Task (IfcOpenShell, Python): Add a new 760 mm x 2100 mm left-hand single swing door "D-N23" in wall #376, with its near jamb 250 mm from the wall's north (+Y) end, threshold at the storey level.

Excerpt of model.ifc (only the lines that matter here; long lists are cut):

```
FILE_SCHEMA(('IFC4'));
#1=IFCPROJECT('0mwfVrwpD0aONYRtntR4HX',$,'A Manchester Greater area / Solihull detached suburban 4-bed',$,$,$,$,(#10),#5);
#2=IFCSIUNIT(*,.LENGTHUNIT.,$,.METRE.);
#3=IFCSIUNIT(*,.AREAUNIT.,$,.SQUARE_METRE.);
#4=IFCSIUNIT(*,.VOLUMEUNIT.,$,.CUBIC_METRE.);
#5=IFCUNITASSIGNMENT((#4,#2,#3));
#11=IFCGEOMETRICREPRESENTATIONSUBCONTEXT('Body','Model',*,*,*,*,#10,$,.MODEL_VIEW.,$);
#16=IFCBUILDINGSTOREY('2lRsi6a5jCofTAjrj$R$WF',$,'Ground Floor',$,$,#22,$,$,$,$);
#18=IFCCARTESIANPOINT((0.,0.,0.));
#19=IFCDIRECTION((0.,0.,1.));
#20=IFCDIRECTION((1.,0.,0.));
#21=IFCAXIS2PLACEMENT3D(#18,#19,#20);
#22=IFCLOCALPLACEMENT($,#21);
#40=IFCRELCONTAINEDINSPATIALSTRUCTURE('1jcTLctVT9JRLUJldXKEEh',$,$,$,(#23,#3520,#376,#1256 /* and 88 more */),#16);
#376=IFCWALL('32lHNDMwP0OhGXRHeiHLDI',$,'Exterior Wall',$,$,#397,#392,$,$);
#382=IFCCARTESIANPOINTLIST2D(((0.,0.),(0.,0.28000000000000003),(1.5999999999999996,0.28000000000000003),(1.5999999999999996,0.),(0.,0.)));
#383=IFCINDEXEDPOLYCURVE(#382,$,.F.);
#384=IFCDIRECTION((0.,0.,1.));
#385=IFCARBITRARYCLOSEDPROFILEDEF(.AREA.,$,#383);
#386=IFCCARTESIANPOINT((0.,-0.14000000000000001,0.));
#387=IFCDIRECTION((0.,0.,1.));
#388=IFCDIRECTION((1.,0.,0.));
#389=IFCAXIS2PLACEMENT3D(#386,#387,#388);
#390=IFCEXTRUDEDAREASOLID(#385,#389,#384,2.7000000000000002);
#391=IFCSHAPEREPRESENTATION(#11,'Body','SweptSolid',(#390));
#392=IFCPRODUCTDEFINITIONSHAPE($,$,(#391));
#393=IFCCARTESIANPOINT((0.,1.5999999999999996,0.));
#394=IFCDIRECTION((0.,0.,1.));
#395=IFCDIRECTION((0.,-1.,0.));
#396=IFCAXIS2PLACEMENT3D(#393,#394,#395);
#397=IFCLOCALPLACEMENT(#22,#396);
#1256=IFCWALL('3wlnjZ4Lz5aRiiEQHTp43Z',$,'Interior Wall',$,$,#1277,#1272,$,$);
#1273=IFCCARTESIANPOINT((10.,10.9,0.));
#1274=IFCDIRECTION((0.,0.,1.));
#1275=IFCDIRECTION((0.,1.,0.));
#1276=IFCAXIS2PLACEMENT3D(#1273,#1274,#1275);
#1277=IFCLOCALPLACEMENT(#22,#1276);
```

```python
import numpy as np
import ifcopenshell
import ifcopenshell.api.feature
import ifcopenshell.api.geometry
import ifcopenshell.api.root
import ifcopenshell.api.spatial
import ifcopenshell.geom
import ifcopenshell.util.element
import ifcopenshell.util.placement
import ifcopenshell.util.representation
import ifcopenshell.util.shape
import ifcopenshell.util.unit

model = ifcopenshell.open("model.ifc")
unit_scale = ifcopenshell.util.unit.calculate_unit_scale(model)
settings = ifcopenshell.geom.settings()


def volume(element):
    """Net volume in cubic metres, openings subtracted."""
    shape = ifcopenshell.geom.create_shape(settings, element)
    return ifcopenshell.util.shape.get_volume(shape.geometry)


wall = model.by_guid("32lHNDMwP0OhGXRHeiHLDI")
storey = ifcopenshell.util.element.get_container(wall, ifc_class="IfcBuildingStorey")
context = ifcopenshell.util.representation.get_context(model, "Model", "Body", "MODEL_VIEW")
before = volume(wall)

width, height, from_end, sill = 0.76, 2.1, 0.25, 0.0  # metres

# The wall runs along its own X axis, and the end named is its -X end.
wall_shape = ifcopenshell.geom.create_shape(settings, wall)
x, y, z = ifcopenshell.util.shape.get_vertices(wall_shape.geometry).T
start = x.min() + from_end
face, thickness = float(y.min()), float(y.max() - y.min())
wall_matrix = ifcopenshell.util.placement.get_local_placement(wall.ObjectPlacement)
level = ifcopenshell.util.placement.get_local_placement(storey.ObjectPlacement)[2, 3]


def in_wall(x, y):
    """Placement at x, y metres in the wall's axes, at sill height."""
    matrix = wall_matrix.copy()
    matrix[:, 3] = wall_matrix @ np.array([x / unit_scale, y / unit_scale, 0.0, 1.0])
    matrix[2, 3] = level + sill / unit_scale
    return matrix


# Opening: a box that overshoots both wall faces by 50 mm.
opening = ifcopenshell.api.root.create_entity(model, ifc_class="IfcOpeningElement", predefined_type="OPENING")
box = ifcopenshell.api.geometry.add_wall_representation(
    model, context=context, length=width, height=height, thickness=thickness + 0.1
)
ifcopenshell.api.geometry.assign_representation(model, product=opening, representation=box)
ifcopenshell.api.geometry.edit_object_placement(model, product=opening, matrix=in_wall(start, face - 0.05), is_si=False)
ifcopenshell.api.feature.add_feature(model, feature=opening, element=wall)

door = ifcopenshell.api.root.create_entity(model, ifc_class="IfcDoor", name="D-N23", predefined_type="DOOR")
door.OverallWidth, door.OverallHeight = width / unit_scale, height / unit_scale
door.OperationType = "SINGLE_SWING_LEFT"
body = ifcopenshell.api.geometry.add_door_representation(
    model,
    context=context,
    overall_width=door.OverallWidth,
    overall_height=door.OverallHeight,
    operation_type="SINGLE_SWING_LEFT",
    lining_properties={"LiningDepth": thickness / unit_scale, "ThresholdDepth": thickness / unit_scale},
)
ifcopenshell.api.geometry.assign_representation(model, product=door, representation=body)
ifcopenshell.api.spatial.assign_container(model, products=[door], relating_structure=storey)
ifcopenshell.api.feature.add_filling(model, opening=opening, element=door)

# The lining spans the wall, so the door starts at the wall face.
ifcopenshell.api.geometry.edit_object_placement(model, product=door, matrix=in_wall(start, face), is_si=False)

after = volume(wall)

print(f"wall volume {before:.3f} -> {after:.3f} m3")

model.write("model-out.ifc")
```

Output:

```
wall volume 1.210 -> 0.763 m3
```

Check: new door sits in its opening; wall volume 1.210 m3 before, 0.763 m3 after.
